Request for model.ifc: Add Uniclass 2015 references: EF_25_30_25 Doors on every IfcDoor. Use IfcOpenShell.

First a look at what the model holds.

```python
import ifcopenshell

model = ifcopenshell.open("model.ifc")
print(model.schema)
print("classifications:", [c.Name for c in model.by_type("IfcClassification")])
for ifc_class in ("IfcDoor", "IfcRoof", "IfcStair", "IfcWall", "IfcWindow"):
    print(ifc_class, len(model.by_type(ifc_class)))
```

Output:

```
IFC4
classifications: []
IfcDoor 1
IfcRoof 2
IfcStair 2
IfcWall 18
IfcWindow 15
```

```python
import ifcopenshell
import ifcopenshell.api.classification

model = ifcopenshell.open("model.ifc")

system = ifcopenshell.api.classification.add_classification(model, classification="Uniclass 2015")

codes = {
    "IfcDoor": ("EF_25_30_25", "Doors"),
}
for ifc_class, (code, name) in codes.items():
    products = model.by_type(ifc_class)
    ifcopenshell.api.classification.add_reference(
        model, products=products, classification=system, identification=code, name=name
    )
    print(code, len(products))

model.write("model_edited.ifc")
```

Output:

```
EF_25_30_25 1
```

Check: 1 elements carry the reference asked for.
